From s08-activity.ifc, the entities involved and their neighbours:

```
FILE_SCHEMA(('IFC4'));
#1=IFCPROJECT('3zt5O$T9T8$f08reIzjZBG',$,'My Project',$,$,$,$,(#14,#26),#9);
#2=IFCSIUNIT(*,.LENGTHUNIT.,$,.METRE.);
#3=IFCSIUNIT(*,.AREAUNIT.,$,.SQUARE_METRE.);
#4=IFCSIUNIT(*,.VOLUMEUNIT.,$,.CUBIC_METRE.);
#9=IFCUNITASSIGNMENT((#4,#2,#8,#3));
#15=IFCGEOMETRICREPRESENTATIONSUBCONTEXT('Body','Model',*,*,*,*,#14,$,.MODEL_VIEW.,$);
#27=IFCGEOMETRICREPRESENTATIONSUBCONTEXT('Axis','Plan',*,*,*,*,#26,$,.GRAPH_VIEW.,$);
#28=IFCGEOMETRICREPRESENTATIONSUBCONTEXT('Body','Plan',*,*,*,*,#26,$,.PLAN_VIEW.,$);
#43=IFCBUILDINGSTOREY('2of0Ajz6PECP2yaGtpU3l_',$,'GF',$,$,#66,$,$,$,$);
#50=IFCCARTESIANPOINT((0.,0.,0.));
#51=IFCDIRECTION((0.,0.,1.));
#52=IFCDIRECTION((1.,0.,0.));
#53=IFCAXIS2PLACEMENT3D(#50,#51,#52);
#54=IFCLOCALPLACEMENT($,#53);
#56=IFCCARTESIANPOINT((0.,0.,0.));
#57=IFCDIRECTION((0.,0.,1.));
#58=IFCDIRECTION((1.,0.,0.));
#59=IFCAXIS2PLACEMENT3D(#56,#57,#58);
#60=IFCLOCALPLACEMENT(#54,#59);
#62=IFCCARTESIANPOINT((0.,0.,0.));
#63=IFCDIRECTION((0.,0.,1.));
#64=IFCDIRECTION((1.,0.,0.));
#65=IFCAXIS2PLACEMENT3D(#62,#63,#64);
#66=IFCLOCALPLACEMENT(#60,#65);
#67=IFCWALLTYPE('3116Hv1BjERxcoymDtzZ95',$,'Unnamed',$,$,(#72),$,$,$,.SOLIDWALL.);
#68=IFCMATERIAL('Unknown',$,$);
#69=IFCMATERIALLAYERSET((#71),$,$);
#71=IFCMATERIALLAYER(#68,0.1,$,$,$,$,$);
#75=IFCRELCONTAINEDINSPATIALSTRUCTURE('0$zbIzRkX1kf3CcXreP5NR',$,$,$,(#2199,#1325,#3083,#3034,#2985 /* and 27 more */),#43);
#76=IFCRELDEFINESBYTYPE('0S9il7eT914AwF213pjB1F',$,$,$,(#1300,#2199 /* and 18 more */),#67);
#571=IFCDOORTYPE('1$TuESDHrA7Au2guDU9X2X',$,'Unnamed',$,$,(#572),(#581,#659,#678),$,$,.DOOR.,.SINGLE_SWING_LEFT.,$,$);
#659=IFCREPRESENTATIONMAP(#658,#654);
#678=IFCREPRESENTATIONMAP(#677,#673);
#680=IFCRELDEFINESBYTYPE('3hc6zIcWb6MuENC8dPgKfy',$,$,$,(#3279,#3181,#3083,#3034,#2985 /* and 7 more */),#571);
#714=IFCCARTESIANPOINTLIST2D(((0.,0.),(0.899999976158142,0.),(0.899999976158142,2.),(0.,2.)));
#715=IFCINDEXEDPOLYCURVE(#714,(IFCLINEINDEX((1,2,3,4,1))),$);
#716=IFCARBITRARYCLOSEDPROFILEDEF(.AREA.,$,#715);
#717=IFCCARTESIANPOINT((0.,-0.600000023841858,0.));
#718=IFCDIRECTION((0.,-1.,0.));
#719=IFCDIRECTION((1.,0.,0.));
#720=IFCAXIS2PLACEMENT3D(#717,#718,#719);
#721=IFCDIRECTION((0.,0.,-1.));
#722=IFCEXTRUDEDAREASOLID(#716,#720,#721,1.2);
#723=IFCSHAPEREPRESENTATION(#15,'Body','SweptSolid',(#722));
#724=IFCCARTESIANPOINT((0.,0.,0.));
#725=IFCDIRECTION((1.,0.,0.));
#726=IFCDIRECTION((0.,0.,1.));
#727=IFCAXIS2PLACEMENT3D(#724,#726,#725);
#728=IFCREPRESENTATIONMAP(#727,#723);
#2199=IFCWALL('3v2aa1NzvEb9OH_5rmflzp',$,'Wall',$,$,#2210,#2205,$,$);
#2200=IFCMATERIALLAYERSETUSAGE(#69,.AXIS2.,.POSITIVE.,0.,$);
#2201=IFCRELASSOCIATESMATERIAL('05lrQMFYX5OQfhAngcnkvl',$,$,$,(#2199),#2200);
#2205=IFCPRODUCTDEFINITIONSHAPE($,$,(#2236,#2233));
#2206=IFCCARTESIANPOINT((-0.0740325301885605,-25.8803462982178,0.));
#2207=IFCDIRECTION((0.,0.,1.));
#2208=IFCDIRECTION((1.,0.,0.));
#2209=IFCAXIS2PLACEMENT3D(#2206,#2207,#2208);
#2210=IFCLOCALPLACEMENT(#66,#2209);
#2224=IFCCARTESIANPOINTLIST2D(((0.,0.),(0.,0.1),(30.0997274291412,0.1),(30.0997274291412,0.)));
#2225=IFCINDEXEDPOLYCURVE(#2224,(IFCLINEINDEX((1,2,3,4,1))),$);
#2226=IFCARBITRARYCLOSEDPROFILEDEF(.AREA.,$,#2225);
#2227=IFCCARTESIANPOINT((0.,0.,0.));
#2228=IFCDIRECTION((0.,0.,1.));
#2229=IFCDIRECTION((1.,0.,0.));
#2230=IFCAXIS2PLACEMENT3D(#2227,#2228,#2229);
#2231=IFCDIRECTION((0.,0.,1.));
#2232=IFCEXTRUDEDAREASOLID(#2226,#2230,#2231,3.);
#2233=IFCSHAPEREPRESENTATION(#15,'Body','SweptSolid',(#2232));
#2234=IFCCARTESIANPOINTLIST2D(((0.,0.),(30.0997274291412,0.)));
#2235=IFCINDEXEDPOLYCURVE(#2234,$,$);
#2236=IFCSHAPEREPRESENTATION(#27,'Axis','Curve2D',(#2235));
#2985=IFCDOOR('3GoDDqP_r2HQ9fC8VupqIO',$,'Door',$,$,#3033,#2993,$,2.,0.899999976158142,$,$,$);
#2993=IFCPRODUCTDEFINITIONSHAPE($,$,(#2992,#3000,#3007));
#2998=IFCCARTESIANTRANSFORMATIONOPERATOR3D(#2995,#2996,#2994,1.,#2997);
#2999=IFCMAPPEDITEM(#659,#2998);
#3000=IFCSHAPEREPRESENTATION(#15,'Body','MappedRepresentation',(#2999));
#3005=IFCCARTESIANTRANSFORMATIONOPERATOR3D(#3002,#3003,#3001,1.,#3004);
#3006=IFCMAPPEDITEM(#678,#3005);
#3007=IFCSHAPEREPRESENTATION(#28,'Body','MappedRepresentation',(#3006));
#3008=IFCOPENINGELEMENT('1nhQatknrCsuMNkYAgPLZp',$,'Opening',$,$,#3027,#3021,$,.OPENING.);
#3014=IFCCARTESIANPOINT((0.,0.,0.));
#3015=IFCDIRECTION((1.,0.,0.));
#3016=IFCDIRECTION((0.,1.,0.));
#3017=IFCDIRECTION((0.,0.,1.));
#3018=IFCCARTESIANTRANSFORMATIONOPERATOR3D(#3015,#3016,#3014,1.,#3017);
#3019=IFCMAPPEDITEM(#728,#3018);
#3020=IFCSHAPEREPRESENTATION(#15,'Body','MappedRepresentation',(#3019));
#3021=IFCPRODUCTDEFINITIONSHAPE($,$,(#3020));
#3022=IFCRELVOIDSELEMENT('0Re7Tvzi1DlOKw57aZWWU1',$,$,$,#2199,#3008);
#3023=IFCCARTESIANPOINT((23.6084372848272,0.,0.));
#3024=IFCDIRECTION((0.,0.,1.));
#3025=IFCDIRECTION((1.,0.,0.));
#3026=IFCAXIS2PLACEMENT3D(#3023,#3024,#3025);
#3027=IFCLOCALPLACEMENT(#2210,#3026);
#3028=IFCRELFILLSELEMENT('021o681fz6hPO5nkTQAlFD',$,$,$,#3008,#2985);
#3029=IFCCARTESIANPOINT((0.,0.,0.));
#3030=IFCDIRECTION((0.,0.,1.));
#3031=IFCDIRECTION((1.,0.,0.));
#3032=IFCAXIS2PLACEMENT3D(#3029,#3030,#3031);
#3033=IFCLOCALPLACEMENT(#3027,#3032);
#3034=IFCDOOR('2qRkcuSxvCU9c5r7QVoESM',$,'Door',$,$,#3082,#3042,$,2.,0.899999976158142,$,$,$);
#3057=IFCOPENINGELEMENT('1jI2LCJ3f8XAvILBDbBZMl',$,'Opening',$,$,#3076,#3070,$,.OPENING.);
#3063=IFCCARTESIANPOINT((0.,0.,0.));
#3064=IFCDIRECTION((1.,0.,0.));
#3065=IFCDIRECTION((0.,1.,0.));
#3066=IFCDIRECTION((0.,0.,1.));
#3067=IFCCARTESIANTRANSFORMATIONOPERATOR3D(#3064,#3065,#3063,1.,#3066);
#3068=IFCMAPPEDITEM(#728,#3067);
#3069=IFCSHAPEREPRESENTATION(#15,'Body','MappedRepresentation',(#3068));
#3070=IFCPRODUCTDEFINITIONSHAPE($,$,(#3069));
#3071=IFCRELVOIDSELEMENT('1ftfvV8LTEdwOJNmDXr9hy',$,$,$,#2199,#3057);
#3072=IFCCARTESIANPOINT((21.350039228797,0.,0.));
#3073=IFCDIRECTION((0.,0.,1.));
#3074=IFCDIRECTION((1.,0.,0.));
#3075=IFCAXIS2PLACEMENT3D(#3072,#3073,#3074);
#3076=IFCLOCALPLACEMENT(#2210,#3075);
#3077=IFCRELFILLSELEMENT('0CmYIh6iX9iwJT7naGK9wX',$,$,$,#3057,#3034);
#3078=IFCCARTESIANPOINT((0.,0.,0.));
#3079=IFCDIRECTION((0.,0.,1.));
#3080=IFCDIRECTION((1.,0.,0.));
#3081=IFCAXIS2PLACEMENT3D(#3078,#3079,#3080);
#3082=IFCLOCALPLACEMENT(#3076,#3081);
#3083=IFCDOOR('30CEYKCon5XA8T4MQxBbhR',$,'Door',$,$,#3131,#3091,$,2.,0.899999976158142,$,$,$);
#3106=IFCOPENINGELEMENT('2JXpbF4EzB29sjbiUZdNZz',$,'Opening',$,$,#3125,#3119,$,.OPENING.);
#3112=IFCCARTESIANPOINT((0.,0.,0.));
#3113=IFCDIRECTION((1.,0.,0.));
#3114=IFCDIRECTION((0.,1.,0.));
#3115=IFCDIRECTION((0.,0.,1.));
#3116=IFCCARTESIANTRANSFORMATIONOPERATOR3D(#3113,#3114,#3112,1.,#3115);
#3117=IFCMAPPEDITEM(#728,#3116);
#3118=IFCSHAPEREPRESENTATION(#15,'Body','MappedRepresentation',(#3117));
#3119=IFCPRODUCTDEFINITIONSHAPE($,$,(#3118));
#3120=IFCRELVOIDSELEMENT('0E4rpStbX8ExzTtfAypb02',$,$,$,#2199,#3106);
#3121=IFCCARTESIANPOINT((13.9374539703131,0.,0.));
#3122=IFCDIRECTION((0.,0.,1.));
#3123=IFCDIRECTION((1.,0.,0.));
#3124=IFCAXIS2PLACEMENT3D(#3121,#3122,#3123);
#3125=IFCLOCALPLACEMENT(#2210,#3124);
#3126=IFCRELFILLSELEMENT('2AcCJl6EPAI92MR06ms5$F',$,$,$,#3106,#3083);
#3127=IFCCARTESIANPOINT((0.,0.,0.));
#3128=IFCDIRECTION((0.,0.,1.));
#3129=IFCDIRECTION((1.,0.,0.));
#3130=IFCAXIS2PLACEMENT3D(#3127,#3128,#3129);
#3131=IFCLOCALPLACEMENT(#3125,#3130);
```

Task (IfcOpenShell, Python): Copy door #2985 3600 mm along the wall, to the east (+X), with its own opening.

```python
import ifcopenshell
import ifcopenshell.api.feature
import ifcopenshell.api.geometry
import ifcopenshell.api.root
import ifcopenshell.geom
import ifcopenshell.util.element
import ifcopenshell.util.placement
import ifcopenshell.util.shape

model = ifcopenshell.open("s08-activity.ifc")
settings = ifcopenshell.geom.settings()


def volume(element):
    """Net volume in cubic metres, openings subtracted."""
    shape = ifcopenshell.geom.create_shape(settings, element)
    return ifcopenshell.util.shape.get_volume(shape.geometry)


door = model.by_guid("3GoDDqP_r2HQ9fC8VupqIO")
opening = door.FillsVoids[0].RelatingOpeningElement
wall = opening.VoidsElements[0].RelatingBuildingElement
before = volume(wall)
shift = ifcopenshell.util.placement.get_local_placement(wall.ObjectPlacement)[:3, 0] * 3.6

# copy_class copies the void relationship, type, container and properties, but no geometry.
new_opening = ifcopenshell.api.root.copy_class(model, product=opening)
new_opening.Representation = ifcopenshell.util.element.copy_deep(
    model, opening.Representation, exclude=["IfcGeometricRepresentationContext", "IfcRepresentationMap"]
)
new_door = ifcopenshell.api.root.copy_class(model, product=door)
new_door.Representation = ifcopenshell.util.element.copy_deep(
    model, door.Representation, exclude=["IfcGeometricRepresentationContext", "IfcRepresentationMap"]
)
ifcopenshell.api.feature.add_filling(model, opening=new_opening, element=new_door)

for old, new in ((opening, new_opening), (door, new_door)):
    matrix = ifcopenshell.util.placement.get_local_placement(old.ObjectPlacement)
    matrix[:3, 3] += shift
    ifcopenshell.api.geometry.edit_object_placement(model, product=new, matrix=matrix, is_si=False)

after = volume(wall)

print(f"wall volume {before:.3f} -> {after:.3f} m3")

model.write("s08-activity_edited.ifc")
```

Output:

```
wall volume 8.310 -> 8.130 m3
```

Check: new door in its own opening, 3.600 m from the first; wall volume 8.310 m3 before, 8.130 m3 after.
